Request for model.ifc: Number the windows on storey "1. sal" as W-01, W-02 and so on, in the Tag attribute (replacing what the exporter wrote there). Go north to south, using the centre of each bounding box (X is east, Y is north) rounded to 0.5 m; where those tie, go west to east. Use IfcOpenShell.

First a look at what the model holds.

```python
import ifcopenshell
import ifcopenshell.util.element
import ifcopenshell.util.placement

model = ifcopenshell.open("model.ifc")
print(model.schema)
storey = next(s for s in model.by_type("IfcBuildingStorey") if s.Name == "1. sal")
windows = [e for e in ifcopenshell.util.element.get_decomposition(storey) if e.is_a("IfcWindow")]
for e in sorted(windows, key=lambda e: e.id()):
    origin = ifcopenshell.util.placement.get_local_placement(e.ObjectPlacement)[:3, 3]
    print(e.id(), e.Tag, e.Name, origin.round(2) + 0.0, sep=" | ")
```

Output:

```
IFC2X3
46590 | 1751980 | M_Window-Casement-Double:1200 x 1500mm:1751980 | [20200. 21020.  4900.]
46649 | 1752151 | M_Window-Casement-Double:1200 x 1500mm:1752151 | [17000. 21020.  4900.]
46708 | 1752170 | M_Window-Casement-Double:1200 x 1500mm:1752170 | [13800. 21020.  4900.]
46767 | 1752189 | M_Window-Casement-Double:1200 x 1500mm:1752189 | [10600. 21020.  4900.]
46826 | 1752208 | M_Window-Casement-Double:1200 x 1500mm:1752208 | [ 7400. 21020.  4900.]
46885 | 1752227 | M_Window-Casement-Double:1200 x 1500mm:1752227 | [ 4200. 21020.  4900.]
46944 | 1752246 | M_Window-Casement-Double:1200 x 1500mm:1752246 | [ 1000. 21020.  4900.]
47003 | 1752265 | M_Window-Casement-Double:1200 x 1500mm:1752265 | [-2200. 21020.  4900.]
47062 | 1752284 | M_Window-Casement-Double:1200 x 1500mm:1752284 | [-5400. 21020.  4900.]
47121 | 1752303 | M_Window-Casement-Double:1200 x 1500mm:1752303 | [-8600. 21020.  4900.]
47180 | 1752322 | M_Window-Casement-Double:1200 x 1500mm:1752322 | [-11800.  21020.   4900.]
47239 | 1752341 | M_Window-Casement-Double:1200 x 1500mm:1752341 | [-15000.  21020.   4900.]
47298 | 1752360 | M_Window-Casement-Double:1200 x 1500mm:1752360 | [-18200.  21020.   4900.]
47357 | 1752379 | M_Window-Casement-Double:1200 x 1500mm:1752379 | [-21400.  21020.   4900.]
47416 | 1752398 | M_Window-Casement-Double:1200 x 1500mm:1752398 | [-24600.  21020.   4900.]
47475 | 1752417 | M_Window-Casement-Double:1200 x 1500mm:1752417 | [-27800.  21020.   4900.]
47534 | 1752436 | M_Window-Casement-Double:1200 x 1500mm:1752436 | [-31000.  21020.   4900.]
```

```python
import ifcopenshell
import ifcopenshell.geom
import ifcopenshell.util.element
import ifcopenshell.util.shape

model = ifcopenshell.open("model.ifc")
settings = ifcopenshell.geom.settings()
settings.set("use-world-coords", True)


def centre(element):
    shape = ifcopenshell.geom.create_shape(settings, element)
    return ifcopenshell.util.shape.get_bbox_centroid(shape.geometry)


storey = next(s for s in model.by_type("IfcBuildingStorey") if s.Name == "1. sal")
windows = [e for e in ifcopenshell.util.element.get_decomposition(storey) if e.is_a("IfcWindow")]

# Insertion points can sit at a corner or the storey origin, so sort by the geometry (in metres).
centres = {e: centre(e) for e in windows}
windows.sort(key=lambda e: (-round(centres[e][1] / 0.5), centres[e][0]))

for i, e in enumerate(windows, start=1):
    number = f"W-{i:02d}"
    e.Tag = number
    print(e.id(), number)

model.write("model_rev.ifc")
```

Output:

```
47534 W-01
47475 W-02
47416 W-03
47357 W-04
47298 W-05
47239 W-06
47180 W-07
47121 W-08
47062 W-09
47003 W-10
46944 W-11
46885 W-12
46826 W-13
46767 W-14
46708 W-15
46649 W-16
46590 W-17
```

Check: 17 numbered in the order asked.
